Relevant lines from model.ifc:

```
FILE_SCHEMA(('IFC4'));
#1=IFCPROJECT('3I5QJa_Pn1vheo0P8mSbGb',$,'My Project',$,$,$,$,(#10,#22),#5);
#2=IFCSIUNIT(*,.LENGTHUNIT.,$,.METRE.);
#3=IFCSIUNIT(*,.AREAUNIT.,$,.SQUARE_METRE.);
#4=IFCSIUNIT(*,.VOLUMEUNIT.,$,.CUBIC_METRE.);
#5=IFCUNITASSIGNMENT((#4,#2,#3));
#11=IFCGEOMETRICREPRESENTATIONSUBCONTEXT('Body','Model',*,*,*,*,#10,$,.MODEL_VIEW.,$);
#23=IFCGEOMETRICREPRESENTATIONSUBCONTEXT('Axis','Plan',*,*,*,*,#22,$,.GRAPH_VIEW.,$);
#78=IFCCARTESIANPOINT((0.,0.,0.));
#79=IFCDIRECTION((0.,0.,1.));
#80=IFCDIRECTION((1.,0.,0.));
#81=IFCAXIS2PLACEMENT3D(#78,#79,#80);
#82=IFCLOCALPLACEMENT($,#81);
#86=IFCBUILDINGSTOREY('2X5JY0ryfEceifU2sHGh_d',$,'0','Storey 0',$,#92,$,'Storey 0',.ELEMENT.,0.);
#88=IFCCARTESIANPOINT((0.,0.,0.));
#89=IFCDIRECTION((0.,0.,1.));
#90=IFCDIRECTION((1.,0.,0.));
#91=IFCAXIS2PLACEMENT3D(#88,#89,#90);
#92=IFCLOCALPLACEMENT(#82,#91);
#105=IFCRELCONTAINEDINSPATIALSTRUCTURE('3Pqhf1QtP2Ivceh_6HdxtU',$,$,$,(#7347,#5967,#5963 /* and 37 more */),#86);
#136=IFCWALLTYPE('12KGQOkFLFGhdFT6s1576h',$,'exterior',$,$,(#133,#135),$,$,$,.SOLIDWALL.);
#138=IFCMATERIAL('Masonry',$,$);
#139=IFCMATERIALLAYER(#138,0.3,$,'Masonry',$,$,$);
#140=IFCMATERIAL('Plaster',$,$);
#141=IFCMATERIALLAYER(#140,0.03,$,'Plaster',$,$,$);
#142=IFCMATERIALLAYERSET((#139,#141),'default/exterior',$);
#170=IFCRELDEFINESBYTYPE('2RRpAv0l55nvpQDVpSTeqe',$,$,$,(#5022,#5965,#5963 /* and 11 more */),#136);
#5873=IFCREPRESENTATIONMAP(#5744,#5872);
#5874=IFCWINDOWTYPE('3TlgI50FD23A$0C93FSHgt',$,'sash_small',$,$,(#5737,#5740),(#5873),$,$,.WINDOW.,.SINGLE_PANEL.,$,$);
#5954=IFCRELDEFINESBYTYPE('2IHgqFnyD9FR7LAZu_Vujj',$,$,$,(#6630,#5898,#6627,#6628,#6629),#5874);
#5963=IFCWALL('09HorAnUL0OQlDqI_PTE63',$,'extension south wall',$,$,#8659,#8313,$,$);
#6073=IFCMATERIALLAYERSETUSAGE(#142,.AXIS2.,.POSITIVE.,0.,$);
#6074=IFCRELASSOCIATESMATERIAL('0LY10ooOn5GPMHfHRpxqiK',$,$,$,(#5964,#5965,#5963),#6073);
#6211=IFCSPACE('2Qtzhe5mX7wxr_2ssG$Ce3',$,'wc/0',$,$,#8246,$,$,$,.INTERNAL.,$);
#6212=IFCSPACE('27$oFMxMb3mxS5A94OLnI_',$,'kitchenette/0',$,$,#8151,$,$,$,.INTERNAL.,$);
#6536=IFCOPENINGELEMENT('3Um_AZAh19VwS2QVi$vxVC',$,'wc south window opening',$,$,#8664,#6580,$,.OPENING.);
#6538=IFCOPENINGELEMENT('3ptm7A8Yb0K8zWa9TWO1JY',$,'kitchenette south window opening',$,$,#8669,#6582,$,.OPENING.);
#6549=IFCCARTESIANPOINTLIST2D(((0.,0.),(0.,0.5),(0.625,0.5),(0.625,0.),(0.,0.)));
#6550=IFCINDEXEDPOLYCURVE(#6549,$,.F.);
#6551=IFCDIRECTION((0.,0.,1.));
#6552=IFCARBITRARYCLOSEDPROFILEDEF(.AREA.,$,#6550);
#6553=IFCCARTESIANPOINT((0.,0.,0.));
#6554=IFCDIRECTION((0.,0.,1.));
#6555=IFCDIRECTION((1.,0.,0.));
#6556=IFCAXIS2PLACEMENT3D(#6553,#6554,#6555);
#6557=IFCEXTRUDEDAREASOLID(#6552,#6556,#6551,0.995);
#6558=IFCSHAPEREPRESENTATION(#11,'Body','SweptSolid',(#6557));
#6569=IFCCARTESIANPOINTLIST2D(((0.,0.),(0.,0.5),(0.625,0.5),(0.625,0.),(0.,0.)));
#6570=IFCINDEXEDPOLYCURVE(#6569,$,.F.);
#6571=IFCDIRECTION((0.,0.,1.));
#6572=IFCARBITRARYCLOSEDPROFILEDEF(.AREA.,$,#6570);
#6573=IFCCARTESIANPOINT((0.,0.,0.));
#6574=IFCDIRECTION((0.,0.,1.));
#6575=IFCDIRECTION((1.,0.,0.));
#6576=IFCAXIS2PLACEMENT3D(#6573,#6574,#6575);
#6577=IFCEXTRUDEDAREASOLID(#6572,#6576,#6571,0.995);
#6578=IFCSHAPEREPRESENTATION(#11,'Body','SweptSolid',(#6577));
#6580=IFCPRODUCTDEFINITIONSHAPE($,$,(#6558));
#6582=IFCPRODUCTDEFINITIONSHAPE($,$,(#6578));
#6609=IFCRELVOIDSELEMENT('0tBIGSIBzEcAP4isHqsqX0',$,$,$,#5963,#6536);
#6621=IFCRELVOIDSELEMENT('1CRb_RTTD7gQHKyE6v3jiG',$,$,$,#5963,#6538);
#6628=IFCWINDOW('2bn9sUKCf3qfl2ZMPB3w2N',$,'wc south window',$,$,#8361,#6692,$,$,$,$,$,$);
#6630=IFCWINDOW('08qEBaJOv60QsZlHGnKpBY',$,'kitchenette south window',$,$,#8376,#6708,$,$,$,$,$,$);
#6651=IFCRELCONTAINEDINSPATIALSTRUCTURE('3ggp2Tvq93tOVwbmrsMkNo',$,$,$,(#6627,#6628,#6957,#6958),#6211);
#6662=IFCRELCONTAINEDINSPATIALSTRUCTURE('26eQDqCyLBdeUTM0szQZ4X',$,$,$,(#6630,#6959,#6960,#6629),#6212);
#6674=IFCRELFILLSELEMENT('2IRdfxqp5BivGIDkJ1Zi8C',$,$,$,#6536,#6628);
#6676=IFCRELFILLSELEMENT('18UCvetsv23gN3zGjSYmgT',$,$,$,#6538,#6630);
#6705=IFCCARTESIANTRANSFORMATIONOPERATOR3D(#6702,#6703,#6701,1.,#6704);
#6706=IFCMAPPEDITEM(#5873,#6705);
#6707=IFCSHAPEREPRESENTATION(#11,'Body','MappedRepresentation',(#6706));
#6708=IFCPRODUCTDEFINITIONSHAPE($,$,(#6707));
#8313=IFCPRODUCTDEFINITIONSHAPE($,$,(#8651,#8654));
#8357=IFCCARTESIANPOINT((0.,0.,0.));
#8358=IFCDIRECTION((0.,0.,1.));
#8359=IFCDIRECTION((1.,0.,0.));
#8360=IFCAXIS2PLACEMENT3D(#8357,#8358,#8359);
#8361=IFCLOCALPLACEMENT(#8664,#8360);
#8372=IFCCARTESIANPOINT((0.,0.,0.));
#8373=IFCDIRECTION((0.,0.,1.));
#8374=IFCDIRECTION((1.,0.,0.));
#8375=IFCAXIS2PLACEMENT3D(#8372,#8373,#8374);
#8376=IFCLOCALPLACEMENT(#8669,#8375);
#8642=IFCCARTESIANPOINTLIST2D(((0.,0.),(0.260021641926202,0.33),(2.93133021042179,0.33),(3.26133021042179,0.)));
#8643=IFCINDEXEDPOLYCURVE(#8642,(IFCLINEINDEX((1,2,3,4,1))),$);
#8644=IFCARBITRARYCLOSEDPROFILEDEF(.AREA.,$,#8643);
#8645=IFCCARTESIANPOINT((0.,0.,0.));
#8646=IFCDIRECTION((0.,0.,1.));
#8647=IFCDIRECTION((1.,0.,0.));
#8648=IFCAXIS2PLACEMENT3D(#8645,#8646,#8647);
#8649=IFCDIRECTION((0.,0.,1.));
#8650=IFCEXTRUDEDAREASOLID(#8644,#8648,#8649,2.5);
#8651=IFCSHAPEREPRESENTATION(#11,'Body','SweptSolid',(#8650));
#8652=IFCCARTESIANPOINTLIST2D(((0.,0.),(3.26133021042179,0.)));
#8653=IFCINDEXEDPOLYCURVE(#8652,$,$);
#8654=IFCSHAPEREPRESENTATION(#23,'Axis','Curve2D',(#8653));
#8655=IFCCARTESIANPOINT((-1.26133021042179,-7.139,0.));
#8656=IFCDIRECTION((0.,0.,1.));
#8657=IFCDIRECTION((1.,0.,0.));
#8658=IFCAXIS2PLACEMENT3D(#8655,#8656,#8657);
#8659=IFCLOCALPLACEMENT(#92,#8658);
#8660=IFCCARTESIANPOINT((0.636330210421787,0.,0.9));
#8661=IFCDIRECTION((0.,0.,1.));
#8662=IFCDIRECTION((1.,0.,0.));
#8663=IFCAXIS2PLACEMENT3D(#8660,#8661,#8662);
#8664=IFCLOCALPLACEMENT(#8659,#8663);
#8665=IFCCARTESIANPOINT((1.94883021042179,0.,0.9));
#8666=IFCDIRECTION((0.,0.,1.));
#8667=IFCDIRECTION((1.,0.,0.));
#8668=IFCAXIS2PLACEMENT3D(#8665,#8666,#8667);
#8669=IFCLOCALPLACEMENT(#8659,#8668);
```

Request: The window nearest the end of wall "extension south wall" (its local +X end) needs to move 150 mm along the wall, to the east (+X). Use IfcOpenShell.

```python
import ifcopenshell
import ifcopenshell.api.geometry
import ifcopenshell.util.placement
import ifcopenshell.util.unit

model = ifcopenshell.open("model.ifc")
unit_scale = ifcopenshell.util.unit.calculate_unit_scale(model)

window = model.by_guid("08qEBaJOv60QsZlHGnKpBY")
opening = window.FillsVoids[0].RelatingOpeningElement
wall = opening.VoidsElements[0].RelatingBuildingElement

wall_matrix = ifcopenshell.util.placement.get_local_placement(wall.ObjectPlacement)
shift = wall_matrix[:3, 0] * 0.15 / unit_scale
before = ifcopenshell.util.placement.get_local_placement(window.ObjectPlacement)[:3, 3].copy()

# The window is placed relative to its opening, so it follows when the opening moves.
matrix = ifcopenshell.util.placement.get_local_placement(opening.ObjectPlacement)
matrix[:3, 3] += shift
ifcopenshell.api.geometry.edit_object_placement(
    model, product=opening, matrix=matrix, is_si=False, should_transform_children=True
)

after = ifcopenshell.util.placement.get_local_placement(window.ObjectPlacement)[:3, 3]
print("window moved by", (after - before).round(3) + 0.0)

model.write("model-out.ifc")
```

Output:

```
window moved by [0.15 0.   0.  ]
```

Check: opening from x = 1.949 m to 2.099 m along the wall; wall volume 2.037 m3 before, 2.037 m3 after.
